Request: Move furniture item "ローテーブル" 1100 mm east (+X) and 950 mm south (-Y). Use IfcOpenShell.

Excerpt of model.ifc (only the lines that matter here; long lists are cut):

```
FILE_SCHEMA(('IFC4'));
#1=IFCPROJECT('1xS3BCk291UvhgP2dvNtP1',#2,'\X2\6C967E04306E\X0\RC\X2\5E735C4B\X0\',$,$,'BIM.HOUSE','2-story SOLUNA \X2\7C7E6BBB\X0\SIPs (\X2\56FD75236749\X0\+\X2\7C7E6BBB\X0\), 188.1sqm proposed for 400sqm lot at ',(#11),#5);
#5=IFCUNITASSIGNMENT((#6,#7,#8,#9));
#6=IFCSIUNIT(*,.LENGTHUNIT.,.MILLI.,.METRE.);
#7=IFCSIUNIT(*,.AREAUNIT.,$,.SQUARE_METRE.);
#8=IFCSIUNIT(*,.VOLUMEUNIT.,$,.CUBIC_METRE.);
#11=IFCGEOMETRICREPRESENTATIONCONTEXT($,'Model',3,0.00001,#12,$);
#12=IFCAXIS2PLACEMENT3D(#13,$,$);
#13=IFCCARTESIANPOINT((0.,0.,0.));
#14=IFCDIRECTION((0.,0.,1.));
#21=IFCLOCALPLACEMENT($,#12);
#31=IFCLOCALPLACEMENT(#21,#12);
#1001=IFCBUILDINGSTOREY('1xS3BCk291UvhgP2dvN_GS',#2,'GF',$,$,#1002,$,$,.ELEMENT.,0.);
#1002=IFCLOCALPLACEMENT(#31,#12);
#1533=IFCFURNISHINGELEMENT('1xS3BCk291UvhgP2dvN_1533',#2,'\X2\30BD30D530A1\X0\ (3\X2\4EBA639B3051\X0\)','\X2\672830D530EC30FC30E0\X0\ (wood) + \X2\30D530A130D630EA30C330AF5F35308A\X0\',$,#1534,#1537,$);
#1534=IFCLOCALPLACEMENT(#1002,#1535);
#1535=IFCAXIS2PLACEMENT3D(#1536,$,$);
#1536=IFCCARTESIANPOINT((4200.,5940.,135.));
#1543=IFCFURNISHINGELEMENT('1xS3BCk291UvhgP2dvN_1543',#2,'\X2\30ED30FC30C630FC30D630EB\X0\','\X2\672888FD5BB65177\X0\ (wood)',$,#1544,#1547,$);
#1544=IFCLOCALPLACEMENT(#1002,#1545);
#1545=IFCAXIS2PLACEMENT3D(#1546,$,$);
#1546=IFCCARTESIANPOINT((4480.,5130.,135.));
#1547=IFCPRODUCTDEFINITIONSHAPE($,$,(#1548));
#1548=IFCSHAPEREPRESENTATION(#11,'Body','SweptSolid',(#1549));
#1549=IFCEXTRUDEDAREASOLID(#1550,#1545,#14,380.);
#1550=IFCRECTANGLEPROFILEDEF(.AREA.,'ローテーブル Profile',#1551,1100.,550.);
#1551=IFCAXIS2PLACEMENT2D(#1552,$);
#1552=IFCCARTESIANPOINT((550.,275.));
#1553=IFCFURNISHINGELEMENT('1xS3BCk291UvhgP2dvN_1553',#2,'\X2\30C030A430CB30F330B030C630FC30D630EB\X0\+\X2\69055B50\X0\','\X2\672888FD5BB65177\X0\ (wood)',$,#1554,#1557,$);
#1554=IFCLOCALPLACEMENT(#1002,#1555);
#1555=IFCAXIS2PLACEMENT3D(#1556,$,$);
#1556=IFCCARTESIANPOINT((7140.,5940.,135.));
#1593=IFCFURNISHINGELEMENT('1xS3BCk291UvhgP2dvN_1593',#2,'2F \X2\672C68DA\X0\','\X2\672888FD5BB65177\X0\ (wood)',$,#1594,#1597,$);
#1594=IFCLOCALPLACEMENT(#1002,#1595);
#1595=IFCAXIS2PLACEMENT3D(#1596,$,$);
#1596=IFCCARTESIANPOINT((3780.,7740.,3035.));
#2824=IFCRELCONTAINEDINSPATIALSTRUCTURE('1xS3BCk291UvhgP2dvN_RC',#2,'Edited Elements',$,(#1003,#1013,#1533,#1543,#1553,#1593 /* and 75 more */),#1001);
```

```python
import ifcopenshell
import ifcopenshell.api.geometry
import ifcopenshell.util.placement
import ifcopenshell.util.unit

model = ifcopenshell.open("model.ifc")
unit_scale = ifcopenshell.util.unit.calculate_unit_scale(model)

item = model.by_id(1543)
matrix = ifcopenshell.util.placement.get_local_placement(item.ObjectPlacement)
matrix[0, 3] += 1.1 / unit_scale
matrix[1, 3] -= 0.95 / unit_scale
ifcopenshell.api.geometry.edit_object_placement(model, product=item, matrix=matrix, is_si=False)

print(ifcopenshell.util.placement.get_local_placement(item.ObjectPlacement).round(3) + 0.0)

model.write("model_updated.ifc")
```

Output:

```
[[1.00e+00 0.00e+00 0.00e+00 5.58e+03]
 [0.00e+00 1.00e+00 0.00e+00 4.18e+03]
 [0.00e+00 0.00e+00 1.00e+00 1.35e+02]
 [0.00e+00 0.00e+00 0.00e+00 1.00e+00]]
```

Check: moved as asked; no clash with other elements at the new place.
